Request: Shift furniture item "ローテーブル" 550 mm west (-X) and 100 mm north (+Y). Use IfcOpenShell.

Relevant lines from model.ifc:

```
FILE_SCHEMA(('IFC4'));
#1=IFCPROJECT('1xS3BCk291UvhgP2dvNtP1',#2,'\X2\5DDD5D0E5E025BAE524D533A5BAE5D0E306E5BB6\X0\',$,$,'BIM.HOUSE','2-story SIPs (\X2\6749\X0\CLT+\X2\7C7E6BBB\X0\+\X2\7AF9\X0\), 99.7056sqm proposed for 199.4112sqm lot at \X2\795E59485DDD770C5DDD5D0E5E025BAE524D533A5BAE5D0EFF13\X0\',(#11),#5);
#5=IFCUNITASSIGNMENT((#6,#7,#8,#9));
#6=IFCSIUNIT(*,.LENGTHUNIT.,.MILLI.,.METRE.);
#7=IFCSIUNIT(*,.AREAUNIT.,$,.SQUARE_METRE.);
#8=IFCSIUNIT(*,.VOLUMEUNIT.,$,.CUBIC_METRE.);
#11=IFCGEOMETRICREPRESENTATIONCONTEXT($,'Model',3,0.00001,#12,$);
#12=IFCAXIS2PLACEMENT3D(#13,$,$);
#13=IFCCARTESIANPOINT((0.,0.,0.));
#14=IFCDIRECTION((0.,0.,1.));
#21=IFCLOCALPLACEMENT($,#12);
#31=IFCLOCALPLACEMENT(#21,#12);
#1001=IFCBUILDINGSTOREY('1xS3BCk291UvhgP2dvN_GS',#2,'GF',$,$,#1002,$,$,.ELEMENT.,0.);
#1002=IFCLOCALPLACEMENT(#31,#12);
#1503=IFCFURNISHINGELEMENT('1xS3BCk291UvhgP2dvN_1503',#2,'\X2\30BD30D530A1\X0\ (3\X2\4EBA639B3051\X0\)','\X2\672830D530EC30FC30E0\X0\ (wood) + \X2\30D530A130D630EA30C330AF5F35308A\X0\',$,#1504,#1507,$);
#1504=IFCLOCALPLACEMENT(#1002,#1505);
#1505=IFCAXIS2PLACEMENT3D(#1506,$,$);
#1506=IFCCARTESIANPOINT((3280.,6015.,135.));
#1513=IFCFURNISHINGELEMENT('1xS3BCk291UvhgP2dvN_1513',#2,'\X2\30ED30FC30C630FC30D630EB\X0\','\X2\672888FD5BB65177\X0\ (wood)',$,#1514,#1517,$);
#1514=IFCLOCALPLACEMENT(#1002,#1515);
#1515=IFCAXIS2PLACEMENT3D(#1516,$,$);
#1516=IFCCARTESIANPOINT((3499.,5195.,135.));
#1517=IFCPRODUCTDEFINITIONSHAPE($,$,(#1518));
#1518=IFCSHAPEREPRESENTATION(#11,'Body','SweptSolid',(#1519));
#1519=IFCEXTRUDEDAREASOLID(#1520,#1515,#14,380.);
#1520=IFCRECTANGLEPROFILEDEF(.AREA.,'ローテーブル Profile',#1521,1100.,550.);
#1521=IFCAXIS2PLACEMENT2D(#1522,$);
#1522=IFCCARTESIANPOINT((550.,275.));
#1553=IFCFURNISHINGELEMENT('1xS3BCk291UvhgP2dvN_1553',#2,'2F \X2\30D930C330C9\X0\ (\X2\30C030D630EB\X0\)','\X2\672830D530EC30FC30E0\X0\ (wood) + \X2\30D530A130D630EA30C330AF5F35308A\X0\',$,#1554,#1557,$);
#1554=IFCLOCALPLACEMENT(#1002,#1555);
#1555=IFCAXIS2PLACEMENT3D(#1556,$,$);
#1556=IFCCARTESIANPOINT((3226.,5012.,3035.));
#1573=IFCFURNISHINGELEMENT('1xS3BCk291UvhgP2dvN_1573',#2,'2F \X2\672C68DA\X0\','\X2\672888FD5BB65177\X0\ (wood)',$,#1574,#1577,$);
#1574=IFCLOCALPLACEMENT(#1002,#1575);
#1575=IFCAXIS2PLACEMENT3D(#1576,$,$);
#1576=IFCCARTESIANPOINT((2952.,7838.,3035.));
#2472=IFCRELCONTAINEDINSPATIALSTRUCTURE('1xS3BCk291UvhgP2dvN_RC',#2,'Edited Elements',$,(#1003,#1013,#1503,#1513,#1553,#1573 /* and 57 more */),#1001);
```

```python
import ifcopenshell
import ifcopenshell.api.geometry
import ifcopenshell.util.placement
import ifcopenshell.util.unit

model = ifcopenshell.open("model.ifc")
unit_scale = ifcopenshell.util.unit.calculate_unit_scale(model)

item = model.by_guid("1xS3BCk291UvhgP2dvN_1513")
matrix = ifcopenshell.util.placement.get_local_placement(item.ObjectPlacement)
matrix[0, 3] -= 0.55 / unit_scale
matrix[1, 3] += 0.1 / unit_scale
ifcopenshell.api.geometry.edit_object_placement(model, product=item, matrix=matrix, is_si=False)

print(ifcopenshell.util.placement.get_local_placement(item.ObjectPlacement).round(3) + 0.0)

model.write("model_updated.ifc")
```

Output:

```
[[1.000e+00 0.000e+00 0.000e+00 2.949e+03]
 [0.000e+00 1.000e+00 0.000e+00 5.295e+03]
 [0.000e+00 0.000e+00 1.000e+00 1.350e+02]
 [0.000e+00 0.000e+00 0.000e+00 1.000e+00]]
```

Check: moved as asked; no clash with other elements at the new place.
